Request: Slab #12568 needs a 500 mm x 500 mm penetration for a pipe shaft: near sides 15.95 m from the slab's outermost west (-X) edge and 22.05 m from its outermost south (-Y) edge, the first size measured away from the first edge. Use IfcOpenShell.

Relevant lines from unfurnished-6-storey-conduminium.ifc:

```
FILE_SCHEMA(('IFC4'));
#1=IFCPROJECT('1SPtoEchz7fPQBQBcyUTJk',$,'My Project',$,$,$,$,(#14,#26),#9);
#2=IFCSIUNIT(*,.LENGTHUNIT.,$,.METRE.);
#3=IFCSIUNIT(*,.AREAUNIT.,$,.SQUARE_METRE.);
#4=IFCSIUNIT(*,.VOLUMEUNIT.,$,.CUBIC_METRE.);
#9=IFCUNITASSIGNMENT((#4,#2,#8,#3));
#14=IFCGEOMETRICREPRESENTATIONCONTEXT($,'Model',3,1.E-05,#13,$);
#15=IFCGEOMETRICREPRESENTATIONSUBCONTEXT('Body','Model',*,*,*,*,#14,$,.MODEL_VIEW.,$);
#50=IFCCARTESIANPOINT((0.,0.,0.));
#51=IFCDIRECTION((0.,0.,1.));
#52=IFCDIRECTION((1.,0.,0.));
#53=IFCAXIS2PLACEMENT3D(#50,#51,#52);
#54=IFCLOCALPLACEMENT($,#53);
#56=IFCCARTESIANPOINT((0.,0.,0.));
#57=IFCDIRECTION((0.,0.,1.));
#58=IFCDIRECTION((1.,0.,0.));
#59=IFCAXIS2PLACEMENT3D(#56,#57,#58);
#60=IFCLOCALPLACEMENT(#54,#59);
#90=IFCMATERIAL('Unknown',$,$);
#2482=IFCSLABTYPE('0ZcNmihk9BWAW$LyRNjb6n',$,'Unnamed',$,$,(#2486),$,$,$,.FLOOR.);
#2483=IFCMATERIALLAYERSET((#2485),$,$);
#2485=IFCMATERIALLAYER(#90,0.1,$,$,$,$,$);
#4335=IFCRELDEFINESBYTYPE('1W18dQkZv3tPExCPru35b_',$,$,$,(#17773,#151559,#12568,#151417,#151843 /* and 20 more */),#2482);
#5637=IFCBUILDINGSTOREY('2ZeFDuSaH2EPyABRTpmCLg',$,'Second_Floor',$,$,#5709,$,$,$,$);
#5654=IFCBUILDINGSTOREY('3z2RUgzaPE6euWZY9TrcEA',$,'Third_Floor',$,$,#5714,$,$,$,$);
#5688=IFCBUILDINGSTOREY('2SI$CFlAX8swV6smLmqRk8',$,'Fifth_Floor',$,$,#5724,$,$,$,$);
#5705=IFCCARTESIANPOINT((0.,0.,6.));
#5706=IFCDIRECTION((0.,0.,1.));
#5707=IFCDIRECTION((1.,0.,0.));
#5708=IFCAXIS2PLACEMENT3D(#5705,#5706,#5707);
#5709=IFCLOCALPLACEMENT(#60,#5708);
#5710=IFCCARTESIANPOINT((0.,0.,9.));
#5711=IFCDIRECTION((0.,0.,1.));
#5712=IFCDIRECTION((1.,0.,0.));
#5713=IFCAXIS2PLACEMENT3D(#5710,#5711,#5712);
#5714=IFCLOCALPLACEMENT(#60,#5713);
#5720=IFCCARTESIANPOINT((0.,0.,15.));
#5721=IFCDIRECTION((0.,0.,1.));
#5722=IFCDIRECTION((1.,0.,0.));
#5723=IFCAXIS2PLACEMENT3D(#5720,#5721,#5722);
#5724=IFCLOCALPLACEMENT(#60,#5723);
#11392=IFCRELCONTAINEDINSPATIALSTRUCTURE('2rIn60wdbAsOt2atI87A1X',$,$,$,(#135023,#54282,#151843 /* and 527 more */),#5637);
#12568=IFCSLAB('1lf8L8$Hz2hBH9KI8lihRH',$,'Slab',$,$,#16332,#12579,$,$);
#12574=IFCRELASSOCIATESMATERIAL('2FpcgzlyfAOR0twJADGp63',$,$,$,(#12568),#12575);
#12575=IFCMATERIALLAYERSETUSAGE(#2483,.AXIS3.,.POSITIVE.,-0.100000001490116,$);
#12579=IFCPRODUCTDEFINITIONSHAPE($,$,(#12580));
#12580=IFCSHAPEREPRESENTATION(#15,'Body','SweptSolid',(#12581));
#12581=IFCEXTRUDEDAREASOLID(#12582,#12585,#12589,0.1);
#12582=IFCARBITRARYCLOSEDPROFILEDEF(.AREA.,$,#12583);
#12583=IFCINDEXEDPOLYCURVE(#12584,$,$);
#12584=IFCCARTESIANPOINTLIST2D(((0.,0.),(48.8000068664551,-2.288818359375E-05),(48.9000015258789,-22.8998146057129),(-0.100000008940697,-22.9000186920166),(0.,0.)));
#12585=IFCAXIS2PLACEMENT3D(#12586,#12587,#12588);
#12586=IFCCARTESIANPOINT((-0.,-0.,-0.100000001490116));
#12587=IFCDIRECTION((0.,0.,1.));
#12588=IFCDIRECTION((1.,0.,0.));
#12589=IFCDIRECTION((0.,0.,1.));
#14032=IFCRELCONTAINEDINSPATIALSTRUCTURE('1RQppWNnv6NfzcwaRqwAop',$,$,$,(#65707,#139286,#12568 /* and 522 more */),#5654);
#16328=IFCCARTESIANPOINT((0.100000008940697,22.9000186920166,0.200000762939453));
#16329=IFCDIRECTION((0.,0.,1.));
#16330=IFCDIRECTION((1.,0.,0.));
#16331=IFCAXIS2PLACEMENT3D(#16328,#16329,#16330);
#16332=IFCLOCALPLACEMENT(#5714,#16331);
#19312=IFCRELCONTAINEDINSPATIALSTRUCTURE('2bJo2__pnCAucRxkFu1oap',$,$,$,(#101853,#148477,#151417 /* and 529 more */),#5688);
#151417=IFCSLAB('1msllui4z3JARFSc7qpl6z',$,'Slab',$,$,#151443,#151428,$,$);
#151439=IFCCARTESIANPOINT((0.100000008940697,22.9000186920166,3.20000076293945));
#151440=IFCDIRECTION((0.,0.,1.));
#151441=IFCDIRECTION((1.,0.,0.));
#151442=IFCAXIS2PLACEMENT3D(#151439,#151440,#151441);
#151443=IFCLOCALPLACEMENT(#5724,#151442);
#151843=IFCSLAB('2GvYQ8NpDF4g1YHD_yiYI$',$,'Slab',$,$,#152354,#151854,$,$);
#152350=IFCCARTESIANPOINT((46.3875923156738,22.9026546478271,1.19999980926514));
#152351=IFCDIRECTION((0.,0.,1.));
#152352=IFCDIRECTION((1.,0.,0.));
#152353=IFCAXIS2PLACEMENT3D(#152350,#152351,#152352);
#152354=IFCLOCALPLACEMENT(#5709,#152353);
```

```python
import numpy as np
import ifcopenshell
import ifcopenshell.api.feature
import ifcopenshell.api.geometry
import ifcopenshell.api.root
import ifcopenshell.geom
import ifcopenshell.util.placement
import ifcopenshell.util.representation
import ifcopenshell.util.shape
import ifcopenshell.util.unit

model = ifcopenshell.open("unfurnished-6-storey-conduminium.ifc")
unit_scale = ifcopenshell.util.unit.calculate_unit_scale(model)
settings = ifcopenshell.geom.settings()


def volume(element):
    """Net volume in cubic metres, openings subtracted."""
    shape = ifcopenshell.geom.create_shape(settings, element)
    return ifcopenshell.util.shape.get_volume(shape.geometry)


slab = model.by_guid("1lf8L8$Hz2hBH9KI8lihRH")
before = volume(slab)

# Extent in the slab's own axes, in metres. The edges named are its -X and -Y sides.
slab_shape = ifcopenshell.geom.create_shape(settings, slab)
vertices = ifcopenshell.util.shape.get_vertices(slab_shape.geometry)
x_min, y_min, bottom = vertices.min(axis=0)
top = vertices[:, 2].max()

opening = ifcopenshell.api.root.create_entity(model, ifc_class="IfcOpeningElement", name="Pipe shaft opening", predefined_type="OPENING")
context = ifcopenshell.util.representation.get_context(model, "Model", "Body", "MODEL_VIEW")
width, depth = 0.5, 0.5
outline = [(0.0, 0.0), (width, 0.0), (width, depth), (0.0, depth), (0.0, 0.0)]
# Overshoot both faces by 50 mm so the cut is clean.
shape = ifcopenshell.api.geometry.add_slab_representation(
    model, context=context, depth=top - bottom + 0.1, polyline=outline
)
ifcopenshell.api.geometry.assign_representation(model, product=opening, representation=shape)

matrix = ifcopenshell.util.placement.get_local_placement(slab.ObjectPlacement)
matrix[:, 3] = matrix @ np.append(np.array([x_min + 15.95, y_min + 22.05, bottom - 0.05]) / unit_scale, 1.0)
ifcopenshell.api.geometry.edit_object_placement(model, product=opening, matrix=matrix, is_si=False)
ifcopenshell.api.feature.add_feature(model, feature=opening, element=slab)

after = volume(slab)

print(f"slab volume {before:.3f} -> {after:.3f} m3")

model.write("unfurnished-6-storey-conduminium_updated.ifc")
```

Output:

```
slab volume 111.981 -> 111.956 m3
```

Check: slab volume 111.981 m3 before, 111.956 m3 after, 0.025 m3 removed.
